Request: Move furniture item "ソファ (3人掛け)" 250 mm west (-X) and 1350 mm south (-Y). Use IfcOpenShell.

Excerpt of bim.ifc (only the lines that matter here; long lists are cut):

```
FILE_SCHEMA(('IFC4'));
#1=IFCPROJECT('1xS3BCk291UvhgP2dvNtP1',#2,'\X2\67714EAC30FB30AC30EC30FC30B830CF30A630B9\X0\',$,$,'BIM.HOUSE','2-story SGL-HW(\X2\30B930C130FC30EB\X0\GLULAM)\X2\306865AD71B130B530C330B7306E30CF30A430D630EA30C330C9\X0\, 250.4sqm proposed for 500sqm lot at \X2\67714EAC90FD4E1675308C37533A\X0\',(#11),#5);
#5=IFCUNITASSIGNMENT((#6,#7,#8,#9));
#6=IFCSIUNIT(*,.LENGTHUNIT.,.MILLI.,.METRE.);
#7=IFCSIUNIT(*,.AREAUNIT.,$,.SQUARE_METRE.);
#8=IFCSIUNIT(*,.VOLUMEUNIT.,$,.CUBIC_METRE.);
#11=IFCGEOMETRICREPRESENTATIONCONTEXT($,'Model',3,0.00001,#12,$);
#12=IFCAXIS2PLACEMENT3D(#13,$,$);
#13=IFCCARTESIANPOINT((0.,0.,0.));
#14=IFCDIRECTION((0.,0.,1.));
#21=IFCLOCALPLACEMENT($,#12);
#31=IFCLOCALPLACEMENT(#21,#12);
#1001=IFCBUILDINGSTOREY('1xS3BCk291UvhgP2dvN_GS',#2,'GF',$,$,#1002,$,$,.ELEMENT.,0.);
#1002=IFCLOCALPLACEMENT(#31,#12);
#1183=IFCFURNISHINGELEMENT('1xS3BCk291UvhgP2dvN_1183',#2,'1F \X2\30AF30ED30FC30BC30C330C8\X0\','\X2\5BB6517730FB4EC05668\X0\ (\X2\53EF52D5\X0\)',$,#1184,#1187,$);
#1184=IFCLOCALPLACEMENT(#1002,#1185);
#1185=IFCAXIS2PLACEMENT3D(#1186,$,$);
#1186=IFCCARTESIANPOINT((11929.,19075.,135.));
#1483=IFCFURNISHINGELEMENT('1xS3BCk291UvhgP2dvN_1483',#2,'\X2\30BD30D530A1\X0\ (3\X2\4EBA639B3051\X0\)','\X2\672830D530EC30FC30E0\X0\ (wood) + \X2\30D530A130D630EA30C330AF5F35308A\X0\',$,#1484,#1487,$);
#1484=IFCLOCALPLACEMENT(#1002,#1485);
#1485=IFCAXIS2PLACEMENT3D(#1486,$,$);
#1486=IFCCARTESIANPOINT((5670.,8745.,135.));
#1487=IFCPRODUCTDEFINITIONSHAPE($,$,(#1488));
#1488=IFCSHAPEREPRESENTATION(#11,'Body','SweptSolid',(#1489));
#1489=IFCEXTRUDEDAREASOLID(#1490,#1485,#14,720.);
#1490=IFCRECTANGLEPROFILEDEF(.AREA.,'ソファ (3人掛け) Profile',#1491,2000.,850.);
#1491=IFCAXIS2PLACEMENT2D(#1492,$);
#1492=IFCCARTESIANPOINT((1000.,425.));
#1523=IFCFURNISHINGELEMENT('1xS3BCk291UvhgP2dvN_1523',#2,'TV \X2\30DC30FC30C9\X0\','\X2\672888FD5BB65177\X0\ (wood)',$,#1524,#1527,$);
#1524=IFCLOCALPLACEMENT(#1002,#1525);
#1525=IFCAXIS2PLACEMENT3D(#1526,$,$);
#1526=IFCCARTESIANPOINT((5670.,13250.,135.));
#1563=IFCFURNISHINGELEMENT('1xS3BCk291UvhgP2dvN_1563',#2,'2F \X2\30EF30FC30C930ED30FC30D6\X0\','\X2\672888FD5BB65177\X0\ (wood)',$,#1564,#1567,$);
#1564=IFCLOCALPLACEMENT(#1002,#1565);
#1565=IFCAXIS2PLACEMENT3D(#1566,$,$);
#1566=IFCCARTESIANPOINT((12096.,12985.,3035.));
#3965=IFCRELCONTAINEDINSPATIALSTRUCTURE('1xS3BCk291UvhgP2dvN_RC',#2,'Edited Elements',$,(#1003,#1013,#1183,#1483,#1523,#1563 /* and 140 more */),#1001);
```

```python
import ifcopenshell
import ifcopenshell.api.geometry
import ifcopenshell.util.placement

model = ifcopenshell.open("bim.ifc")

item = model.by_guid("1xS3BCk291UvhgP2dvN_1483")
matrix = ifcopenshell.util.placement.get_local_placement(item.ObjectPlacement)
matrix[0, 3] -= 250.0
matrix[1, 3] -= 1350.0
ifcopenshell.api.geometry.edit_object_placement(model, product=item, matrix=matrix, is_si=False)

print(ifcopenshell.util.placement.get_local_placement(item.ObjectPlacement).round(3) + 0.0)

model.write("bim_updated.ifc")
```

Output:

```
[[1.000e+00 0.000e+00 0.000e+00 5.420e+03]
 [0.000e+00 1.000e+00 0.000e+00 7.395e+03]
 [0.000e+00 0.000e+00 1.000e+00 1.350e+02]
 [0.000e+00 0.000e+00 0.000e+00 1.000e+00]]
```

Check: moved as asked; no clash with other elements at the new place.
